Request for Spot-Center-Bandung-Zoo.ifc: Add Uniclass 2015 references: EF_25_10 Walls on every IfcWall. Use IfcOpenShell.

First a look at what the model holds.

```python
import ifcopenshell

model = ifcopenshell.open("Spot-Center-Bandung-Zoo.ifc")
print(model.schema)
print("classifications:", [c.Name for c in model.by_type("IfcClassification")])
for ifc_class in ("IfcDoor", "IfcRoof", "IfcStair", "IfcWall", "IfcWindow"):
    print(ifc_class, len(model.by_type(ifc_class)))
```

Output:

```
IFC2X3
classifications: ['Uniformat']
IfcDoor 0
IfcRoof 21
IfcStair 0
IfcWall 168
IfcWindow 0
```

```python
import ifcopenshell
import ifcopenshell.api.classification

model = ifcopenshell.open("Spot-Center-Bandung-Zoo.ifc")

# IFC2X3 requires Source and Edition and has no link from the project to the system.
system = model.create_entity("IfcClassification", Source="NBS", Edition="2015", Name="Uniclass 2015")

codes = {
    "IfcWall": ("EF_25_10", "Walls"),
}
for ifc_class, (code, name) in codes.items():
    products = model.by_type(ifc_class)
    ifcopenshell.api.classification.add_reference(
        model, products=products, classification=system, identification=code, name=name
    )
    print(code, len(products))

model.write("Spot-Center-Bandung-Zoo_v2.ifc")
```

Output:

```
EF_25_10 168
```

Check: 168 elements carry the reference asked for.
